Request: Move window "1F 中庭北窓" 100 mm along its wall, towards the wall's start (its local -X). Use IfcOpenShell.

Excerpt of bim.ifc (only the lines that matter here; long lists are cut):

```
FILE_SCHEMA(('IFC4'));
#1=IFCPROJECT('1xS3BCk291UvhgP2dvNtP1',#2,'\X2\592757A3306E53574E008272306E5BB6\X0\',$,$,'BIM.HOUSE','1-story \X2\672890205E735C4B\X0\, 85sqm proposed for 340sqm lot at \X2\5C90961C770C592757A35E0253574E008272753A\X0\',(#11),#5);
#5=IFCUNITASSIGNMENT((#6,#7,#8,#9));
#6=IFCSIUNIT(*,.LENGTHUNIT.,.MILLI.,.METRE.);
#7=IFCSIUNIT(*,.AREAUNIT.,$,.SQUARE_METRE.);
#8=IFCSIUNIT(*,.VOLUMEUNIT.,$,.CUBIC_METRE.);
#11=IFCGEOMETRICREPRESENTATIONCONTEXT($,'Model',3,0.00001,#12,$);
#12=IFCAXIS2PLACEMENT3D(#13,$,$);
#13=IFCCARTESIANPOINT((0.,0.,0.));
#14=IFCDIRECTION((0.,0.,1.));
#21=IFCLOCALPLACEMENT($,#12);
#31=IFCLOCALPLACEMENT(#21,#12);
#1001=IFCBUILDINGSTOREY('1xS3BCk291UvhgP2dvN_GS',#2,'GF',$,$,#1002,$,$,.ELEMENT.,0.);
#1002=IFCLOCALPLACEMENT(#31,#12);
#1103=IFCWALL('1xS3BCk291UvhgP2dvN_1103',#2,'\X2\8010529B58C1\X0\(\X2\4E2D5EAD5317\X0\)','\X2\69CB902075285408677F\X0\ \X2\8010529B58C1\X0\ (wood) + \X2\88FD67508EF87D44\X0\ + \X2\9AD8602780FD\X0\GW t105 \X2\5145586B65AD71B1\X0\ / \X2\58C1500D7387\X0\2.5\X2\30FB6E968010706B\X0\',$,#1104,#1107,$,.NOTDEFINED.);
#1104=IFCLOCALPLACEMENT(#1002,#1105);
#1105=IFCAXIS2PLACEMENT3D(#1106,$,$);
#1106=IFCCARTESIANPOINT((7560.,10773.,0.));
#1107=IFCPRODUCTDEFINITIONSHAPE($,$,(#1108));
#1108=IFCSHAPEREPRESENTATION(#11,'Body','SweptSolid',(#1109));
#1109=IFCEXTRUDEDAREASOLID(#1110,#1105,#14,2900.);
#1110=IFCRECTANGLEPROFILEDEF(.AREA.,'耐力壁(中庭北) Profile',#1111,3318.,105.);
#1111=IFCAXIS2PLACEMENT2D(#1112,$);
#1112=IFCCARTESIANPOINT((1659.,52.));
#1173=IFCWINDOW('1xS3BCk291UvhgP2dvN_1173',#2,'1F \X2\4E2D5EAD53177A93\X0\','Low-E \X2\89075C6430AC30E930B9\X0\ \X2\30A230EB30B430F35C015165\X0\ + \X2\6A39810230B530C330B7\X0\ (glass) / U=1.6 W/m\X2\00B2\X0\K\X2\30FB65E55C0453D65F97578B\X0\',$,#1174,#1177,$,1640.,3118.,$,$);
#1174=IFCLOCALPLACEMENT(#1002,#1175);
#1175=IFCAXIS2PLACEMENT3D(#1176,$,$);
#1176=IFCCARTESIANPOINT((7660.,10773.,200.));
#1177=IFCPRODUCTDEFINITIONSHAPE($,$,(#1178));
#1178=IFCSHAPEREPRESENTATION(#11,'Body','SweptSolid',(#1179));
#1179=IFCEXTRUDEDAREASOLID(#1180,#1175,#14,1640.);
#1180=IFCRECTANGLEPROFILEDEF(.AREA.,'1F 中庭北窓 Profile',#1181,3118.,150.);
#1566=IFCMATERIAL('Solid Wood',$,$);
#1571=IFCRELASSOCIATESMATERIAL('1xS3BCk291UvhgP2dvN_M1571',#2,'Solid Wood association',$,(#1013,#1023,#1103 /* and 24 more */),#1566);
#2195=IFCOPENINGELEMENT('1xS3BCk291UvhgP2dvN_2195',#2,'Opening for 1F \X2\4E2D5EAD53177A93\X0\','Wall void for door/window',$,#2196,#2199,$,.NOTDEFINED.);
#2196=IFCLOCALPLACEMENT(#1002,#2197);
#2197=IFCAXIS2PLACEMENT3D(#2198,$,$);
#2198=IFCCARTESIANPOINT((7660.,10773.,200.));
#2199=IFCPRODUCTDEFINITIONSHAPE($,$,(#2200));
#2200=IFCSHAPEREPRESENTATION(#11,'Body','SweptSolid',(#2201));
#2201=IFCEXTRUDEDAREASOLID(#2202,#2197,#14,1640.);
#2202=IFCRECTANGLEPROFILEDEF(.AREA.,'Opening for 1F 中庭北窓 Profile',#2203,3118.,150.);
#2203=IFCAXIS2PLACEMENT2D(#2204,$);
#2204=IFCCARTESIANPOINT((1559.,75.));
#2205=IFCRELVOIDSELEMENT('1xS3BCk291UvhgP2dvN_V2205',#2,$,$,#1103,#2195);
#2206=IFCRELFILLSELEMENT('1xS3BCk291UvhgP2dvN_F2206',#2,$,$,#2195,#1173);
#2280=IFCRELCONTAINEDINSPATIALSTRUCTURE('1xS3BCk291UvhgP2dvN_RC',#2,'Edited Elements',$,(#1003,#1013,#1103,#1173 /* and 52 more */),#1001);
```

```python
import ifcopenshell
import ifcopenshell.api.geometry
import ifcopenshell.util.placement
import ifcopenshell.util.unit

model = ifcopenshell.open("bim.ifc")
unit_scale = ifcopenshell.util.unit.calculate_unit_scale(model)

window = model.by_guid("1xS3BCk291UvhgP2dvN_1173")
opening = window.FillsVoids[0].RelatingOpeningElement
wall = opening.VoidsElements[0].RelatingBuildingElement

wall_matrix = ifcopenshell.util.placement.get_local_placement(wall.ObjectPlacement)
shift = wall_matrix[:3, 0] * -0.1 / unit_scale
before = ifcopenshell.util.placement.get_local_placement(window.ObjectPlacement)[:3, 3].copy()

# The window is not placed relative to its opening, so move both.
for product in (opening, window):
    matrix = ifcopenshell.util.placement.get_local_placement(product.ObjectPlacement)
    matrix[:3, 3] += shift
    ifcopenshell.api.geometry.edit_object_placement(model, product=product, matrix=matrix, is_si=False)

after = ifcopenshell.util.placement.get_local_placement(window.ObjectPlacement)[:3, 3]
print("window moved by", (after - before).round(3) + 0.0)

model.write("bim_v2.ifc")
```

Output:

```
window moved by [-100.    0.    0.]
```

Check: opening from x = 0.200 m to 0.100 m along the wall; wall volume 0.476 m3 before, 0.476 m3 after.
